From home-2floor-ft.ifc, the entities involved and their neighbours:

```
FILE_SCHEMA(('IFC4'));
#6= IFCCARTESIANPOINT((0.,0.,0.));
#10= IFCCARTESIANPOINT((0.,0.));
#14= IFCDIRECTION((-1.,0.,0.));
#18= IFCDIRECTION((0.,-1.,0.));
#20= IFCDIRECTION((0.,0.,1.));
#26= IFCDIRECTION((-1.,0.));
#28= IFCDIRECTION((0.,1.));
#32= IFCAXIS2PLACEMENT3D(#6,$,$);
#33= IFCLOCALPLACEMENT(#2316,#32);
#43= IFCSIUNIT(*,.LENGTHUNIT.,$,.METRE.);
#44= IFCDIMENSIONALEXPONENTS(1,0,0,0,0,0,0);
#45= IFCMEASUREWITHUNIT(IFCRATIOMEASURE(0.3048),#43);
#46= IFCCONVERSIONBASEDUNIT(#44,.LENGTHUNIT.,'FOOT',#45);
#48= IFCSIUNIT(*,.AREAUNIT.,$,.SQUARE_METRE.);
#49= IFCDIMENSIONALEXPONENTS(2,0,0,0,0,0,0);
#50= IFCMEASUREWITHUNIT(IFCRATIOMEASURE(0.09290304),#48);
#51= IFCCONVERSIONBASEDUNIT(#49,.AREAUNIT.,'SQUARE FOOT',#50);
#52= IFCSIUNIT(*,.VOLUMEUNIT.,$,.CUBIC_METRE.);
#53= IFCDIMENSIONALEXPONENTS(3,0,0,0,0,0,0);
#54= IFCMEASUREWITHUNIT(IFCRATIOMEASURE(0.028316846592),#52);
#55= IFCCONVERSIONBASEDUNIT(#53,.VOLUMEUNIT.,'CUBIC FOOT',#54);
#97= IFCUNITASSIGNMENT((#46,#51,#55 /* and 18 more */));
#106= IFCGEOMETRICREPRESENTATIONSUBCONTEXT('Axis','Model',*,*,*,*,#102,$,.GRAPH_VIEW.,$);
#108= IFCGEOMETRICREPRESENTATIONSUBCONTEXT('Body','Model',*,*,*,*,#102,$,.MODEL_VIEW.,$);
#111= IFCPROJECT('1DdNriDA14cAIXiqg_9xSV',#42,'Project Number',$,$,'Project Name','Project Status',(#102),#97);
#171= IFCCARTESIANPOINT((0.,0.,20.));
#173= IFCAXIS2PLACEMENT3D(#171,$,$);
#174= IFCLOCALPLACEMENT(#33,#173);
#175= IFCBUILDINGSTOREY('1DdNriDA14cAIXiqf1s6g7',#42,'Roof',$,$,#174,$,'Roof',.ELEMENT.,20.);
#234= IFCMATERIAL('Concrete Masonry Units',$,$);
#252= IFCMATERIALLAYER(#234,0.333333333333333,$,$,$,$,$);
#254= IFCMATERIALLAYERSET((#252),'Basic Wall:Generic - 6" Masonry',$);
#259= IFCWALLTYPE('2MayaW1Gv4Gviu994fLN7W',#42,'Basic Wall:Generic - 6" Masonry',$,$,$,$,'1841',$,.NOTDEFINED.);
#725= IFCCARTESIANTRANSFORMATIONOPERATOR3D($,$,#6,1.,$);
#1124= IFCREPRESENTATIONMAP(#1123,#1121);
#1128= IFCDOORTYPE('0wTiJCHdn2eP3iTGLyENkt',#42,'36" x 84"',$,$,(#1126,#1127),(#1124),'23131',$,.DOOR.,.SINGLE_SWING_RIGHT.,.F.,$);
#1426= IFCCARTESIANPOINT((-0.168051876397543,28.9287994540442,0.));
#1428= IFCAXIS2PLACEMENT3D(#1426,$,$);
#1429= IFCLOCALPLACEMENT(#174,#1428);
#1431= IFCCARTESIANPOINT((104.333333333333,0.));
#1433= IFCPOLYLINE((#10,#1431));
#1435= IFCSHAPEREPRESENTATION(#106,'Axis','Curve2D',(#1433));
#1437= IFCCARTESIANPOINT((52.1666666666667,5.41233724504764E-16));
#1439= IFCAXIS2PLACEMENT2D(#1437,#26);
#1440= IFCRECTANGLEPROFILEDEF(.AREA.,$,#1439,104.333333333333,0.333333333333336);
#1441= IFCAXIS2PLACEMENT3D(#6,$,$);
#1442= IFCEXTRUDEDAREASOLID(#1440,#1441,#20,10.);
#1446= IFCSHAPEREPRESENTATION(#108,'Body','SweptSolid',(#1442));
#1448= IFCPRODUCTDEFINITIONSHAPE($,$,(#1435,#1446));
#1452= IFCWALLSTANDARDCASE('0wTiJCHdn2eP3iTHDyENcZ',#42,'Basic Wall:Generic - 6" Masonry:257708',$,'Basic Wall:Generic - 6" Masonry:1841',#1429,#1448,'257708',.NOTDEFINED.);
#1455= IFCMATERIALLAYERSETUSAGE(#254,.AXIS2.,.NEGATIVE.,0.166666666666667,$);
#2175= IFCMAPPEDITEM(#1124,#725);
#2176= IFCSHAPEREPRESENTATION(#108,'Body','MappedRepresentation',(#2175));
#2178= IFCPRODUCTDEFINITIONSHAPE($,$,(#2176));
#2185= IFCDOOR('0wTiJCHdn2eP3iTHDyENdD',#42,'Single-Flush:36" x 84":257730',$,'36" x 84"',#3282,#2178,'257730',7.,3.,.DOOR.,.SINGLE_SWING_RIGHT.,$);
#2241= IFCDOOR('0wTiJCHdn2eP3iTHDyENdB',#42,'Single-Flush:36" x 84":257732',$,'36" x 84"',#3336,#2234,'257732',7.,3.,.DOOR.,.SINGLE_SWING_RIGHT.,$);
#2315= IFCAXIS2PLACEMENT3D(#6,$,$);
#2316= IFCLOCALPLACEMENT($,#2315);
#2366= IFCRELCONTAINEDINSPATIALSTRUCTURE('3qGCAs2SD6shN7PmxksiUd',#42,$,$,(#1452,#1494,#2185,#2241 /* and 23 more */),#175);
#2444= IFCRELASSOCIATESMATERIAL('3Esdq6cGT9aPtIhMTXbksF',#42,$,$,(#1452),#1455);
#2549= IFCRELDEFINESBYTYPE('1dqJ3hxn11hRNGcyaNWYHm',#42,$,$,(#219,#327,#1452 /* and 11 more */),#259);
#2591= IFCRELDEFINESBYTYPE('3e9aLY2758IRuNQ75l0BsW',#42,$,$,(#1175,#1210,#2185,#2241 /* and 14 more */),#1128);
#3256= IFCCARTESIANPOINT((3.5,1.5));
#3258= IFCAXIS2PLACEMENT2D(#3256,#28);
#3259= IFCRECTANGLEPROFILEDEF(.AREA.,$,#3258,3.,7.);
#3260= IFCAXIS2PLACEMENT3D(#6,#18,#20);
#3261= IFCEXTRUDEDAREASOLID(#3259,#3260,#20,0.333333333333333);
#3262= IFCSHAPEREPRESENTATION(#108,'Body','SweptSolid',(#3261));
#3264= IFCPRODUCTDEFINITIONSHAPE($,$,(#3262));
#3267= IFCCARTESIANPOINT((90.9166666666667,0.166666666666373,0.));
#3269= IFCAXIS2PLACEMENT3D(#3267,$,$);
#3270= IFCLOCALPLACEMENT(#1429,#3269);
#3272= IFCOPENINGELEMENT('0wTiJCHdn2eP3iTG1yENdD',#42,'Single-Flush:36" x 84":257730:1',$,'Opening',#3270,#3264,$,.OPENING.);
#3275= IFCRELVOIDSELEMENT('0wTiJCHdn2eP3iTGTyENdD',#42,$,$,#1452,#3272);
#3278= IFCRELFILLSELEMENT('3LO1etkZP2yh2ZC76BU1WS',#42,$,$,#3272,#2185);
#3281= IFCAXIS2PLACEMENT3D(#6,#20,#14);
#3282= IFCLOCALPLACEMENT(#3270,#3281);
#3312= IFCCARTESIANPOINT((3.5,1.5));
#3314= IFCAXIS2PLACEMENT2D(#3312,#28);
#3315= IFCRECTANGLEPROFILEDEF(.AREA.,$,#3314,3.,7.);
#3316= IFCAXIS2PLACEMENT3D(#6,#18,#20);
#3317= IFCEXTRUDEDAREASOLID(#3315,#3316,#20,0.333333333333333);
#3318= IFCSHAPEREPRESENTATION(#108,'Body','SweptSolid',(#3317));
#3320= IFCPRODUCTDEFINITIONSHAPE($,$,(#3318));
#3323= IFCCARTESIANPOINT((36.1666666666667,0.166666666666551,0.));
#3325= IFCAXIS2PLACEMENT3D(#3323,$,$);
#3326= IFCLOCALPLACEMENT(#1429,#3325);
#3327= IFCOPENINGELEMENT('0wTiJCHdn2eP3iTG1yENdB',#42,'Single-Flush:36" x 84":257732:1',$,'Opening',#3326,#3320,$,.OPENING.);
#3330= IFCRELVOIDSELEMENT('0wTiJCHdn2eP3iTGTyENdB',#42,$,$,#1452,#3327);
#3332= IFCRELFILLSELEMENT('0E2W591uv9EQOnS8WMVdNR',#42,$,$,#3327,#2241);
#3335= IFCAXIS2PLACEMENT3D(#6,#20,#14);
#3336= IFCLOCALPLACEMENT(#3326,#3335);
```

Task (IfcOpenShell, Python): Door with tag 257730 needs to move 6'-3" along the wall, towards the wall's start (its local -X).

```python
import ifcopenshell
import ifcopenshell.api.geometry
import ifcopenshell.util.placement
import ifcopenshell.util.unit

model = ifcopenshell.open("home-2floor-ft.ifc")
unit_scale = ifcopenshell.util.unit.calculate_unit_scale(model)

door = model.by_guid("0wTiJCHdn2eP3iTHDyENdD")
opening = door.FillsVoids[0].RelatingOpeningElement
wall = opening.VoidsElements[0].RelatingBuildingElement

wall_matrix = ifcopenshell.util.placement.get_local_placement(wall.ObjectPlacement)
shift = wall_matrix[:3, 0] * -75 * 0.0254 / unit_scale
before = ifcopenshell.util.placement.get_local_placement(door.ObjectPlacement)[:3, 3].copy()

# The door is placed relative to its opening, so it follows when the opening moves.
matrix = ifcopenshell.util.placement.get_local_placement(opening.ObjectPlacement)
matrix[:3, 3] += shift
ifcopenshell.api.geometry.edit_object_placement(
    model, product=opening, matrix=matrix, is_si=False, should_transform_children=True
)

after = ifcopenshell.util.placement.get_local_placement(door.ObjectPlacement)[:3, 3]
print("door moved by", (after - before).round(3) + 0.0)

model.write("home-2floor-ft_edited.ifc")
```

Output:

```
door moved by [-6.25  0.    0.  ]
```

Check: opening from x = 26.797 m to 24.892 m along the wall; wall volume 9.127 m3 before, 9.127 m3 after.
